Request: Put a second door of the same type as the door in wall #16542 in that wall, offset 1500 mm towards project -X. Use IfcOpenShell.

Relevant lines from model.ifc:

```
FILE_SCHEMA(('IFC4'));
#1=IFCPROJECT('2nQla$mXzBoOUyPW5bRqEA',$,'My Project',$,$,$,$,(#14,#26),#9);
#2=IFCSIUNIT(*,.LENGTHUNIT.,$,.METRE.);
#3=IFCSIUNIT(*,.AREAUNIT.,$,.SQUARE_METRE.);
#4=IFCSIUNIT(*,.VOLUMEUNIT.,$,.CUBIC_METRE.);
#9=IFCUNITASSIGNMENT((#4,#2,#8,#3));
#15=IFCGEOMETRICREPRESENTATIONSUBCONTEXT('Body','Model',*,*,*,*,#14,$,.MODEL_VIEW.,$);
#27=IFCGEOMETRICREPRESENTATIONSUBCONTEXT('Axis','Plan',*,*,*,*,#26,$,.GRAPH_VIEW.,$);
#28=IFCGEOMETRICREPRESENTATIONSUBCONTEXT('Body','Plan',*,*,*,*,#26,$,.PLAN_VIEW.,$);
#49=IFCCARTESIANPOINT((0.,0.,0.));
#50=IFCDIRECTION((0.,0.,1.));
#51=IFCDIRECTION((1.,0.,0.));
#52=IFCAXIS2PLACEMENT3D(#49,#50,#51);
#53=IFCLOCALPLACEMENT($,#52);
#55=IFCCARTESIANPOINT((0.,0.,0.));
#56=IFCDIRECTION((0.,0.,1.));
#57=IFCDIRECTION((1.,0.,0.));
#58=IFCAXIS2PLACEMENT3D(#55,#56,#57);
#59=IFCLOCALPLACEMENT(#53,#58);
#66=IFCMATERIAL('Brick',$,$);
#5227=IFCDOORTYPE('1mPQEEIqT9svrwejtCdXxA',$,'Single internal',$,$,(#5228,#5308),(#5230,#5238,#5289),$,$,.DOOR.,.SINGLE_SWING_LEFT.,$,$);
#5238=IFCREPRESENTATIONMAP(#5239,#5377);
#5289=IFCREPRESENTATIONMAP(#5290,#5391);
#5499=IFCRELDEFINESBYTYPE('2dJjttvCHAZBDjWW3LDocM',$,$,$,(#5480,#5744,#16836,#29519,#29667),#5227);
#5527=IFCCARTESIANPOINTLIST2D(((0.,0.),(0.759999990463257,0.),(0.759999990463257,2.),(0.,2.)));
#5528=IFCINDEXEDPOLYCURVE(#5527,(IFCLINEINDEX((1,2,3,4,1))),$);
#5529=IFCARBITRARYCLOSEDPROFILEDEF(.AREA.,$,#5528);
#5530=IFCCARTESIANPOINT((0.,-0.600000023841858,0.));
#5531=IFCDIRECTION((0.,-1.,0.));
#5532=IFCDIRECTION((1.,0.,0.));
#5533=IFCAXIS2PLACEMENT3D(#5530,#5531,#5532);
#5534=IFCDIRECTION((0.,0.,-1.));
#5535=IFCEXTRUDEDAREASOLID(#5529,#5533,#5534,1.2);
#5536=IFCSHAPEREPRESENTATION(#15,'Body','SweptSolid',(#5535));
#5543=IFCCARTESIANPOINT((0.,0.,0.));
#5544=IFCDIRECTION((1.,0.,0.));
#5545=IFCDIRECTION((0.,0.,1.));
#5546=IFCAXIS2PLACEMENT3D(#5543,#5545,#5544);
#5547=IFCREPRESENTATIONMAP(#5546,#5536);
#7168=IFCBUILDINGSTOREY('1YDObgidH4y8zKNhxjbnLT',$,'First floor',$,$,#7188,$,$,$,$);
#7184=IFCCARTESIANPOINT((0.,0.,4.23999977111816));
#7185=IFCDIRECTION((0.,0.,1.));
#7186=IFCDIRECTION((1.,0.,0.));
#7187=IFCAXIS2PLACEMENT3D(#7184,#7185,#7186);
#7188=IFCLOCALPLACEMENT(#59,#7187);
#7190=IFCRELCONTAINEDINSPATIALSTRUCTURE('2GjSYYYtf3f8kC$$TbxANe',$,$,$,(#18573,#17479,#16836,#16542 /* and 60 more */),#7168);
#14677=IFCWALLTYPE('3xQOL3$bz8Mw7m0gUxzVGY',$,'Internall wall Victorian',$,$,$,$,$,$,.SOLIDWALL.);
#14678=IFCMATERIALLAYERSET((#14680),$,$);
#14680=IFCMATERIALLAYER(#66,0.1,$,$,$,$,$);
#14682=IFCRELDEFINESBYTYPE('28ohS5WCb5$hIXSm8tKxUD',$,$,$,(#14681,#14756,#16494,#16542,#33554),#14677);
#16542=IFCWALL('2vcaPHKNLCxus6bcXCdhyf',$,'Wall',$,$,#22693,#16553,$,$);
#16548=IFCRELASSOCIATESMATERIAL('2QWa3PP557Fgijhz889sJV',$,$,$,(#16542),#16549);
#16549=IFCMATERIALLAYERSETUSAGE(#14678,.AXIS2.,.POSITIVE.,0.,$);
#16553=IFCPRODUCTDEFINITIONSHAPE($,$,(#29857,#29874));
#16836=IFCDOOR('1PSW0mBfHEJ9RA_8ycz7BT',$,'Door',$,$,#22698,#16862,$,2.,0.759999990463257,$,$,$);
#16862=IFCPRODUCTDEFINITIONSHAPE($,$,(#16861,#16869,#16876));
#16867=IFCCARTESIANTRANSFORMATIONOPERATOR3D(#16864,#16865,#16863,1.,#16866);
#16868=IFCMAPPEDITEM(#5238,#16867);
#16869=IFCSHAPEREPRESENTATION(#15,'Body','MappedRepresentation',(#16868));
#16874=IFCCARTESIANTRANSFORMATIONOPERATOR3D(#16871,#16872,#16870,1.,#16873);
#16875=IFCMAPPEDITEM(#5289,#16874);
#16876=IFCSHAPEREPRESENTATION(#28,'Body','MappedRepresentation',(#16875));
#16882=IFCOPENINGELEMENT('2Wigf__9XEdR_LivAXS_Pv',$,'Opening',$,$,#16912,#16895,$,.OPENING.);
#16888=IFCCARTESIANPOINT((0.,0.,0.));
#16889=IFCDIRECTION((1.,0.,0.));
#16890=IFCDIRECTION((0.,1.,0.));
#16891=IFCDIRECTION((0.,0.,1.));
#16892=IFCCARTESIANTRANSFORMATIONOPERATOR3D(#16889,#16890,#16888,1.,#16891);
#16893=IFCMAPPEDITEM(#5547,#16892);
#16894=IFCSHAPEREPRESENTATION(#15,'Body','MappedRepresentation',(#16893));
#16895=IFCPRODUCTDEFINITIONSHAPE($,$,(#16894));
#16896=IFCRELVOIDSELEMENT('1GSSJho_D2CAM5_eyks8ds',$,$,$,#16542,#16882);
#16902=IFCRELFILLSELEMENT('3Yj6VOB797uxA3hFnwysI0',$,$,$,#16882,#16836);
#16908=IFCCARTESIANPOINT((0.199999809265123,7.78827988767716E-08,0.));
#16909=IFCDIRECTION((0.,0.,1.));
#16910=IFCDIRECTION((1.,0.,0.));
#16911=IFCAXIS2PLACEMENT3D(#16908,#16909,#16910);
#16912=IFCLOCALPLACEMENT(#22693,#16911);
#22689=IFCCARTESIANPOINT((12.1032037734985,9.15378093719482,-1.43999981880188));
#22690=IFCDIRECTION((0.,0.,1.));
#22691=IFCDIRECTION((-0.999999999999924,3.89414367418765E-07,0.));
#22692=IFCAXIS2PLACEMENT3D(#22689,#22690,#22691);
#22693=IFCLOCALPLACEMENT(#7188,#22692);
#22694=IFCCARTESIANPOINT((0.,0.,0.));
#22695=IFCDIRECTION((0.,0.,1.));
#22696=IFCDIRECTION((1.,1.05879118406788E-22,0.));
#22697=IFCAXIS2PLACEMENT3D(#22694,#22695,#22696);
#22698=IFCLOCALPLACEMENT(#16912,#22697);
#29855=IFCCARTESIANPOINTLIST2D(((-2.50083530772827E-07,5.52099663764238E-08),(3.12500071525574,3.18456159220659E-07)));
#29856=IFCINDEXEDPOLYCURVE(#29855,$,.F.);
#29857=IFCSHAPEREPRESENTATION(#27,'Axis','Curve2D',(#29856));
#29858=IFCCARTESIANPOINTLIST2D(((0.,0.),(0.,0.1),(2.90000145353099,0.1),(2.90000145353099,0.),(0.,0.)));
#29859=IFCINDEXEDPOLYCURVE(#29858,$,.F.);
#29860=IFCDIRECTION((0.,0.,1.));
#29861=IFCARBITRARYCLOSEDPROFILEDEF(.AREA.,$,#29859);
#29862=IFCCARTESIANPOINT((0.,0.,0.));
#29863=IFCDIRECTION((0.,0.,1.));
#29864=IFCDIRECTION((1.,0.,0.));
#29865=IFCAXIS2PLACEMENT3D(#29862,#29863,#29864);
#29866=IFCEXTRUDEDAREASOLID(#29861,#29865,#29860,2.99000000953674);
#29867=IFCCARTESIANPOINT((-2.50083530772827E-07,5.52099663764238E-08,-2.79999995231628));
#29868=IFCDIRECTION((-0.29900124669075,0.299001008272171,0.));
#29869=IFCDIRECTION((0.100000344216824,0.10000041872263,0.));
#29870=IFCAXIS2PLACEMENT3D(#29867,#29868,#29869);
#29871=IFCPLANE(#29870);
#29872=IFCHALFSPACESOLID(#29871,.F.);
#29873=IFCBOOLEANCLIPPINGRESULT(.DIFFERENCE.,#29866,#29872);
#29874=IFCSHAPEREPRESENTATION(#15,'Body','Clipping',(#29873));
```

```python
import ifcopenshell
import ifcopenshell.api.feature
import ifcopenshell.api.geometry
import ifcopenshell.api.root
import ifcopenshell.geom
import ifcopenshell.util.element
import ifcopenshell.util.placement
import ifcopenshell.util.shape
import ifcopenshell.util.unit

model = ifcopenshell.open("model.ifc")
unit_scale = ifcopenshell.util.unit.calculate_unit_scale(model)
settings = ifcopenshell.geom.settings()


def volume(element):
    """Net volume in cubic metres, openings subtracted."""
    shape = ifcopenshell.geom.create_shape(settings, element)
    return ifcopenshell.util.shape.get_volume(shape.geometry)


door = model.by_guid("1PSW0mBfHEJ9RA_8ycz7BT")
opening = door.FillsVoids[0].RelatingOpeningElement
wall = opening.VoidsElements[0].RelatingBuildingElement
before = volume(wall)
shift = ifcopenshell.util.placement.get_local_placement(wall.ObjectPlacement)[:3, 0] * 1.5 / unit_scale

# copy_class copies the void relationship, type, container and properties, but no geometry.
new_opening = ifcopenshell.api.root.copy_class(model, product=opening)
new_opening.Representation = ifcopenshell.util.element.copy_deep(
    model, opening.Representation, exclude=["IfcGeometricRepresentationContext", "IfcRepresentationMap"]
)
new_door = ifcopenshell.api.root.copy_class(model, product=door)
new_door.Representation = ifcopenshell.util.element.copy_deep(
    model, door.Representation, exclude=["IfcGeometricRepresentationContext", "IfcRepresentationMap"]
)
ifcopenshell.api.feature.add_filling(model, opening=new_opening, element=new_door)

for old, new in ((opening, new_opening), (door, new_door)):
    matrix = ifcopenshell.util.placement.get_local_placement(old.ObjectPlacement)
    matrix[:3, 3] += shift
    ifcopenshell.api.geometry.edit_object_placement(model, product=new, matrix=matrix, is_si=False)

after = volume(wall)

print(f"wall volume {before:.3f} -> {after:.3f} m3")

model.write("model_v2.ifc")
```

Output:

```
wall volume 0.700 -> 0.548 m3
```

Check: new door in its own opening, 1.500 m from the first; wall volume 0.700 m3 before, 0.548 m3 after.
